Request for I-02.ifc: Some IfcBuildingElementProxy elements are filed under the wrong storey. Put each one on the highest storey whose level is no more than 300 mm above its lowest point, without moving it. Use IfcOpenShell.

First a look at what the model holds.

```python
import ifcopenshell
import ifcopenshell.util.element
import ifcopenshell.util.placement

model = ifcopenshell.open("I-02.ifc")
print(model.schema)
for storey in model.by_type("IfcBuildingStorey"):
    level = ifcopenshell.util.placement.get_storey_elevation(storey)
    count = sum(e.is_a("IfcBuildingElementProxy") for e in ifcopenshell.util.element.get_contained(storey))
    print(storey.id(), storey.Name, round(level, 3), count, sep=" | ")
```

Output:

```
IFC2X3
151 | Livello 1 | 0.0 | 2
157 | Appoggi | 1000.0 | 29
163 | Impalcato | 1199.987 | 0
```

```python
import ifcopenshell
import ifcopenshell.api.spatial
import ifcopenshell.geom
import ifcopenshell.util.element
import ifcopenshell.util.placement
import ifcopenshell.util.shape
import ifcopenshell.util.unit

model = ifcopenshell.open("I-02.ifc")
unit_scale = ifcopenshell.util.unit.calculate_unit_scale(model)
settings = ifcopenshell.geom.settings()

levels = sorted(
    ((ifcopenshell.util.placement.get_storey_elevation(s) * unit_scale, s) for s in model.by_type("IfcBuildingStorey")),
    key=lambda pair: pair[0],
)

for e in model.by_type("IfcBuildingElementProxy"):
    current = e.ContainedInStructure[0].RelatingStructure if e.ContainedInStructure else None
    if current is None or not current.is_a("IfcBuildingStorey"):
        continue
    shape = ifcopenshell.geom.create_shape(settings, e)
    bottom = ifcopenshell.util.shape.get_shape_bottom_elevation(shape, shape.geometry)
    below = [s for level, s in levels if level <= bottom + 0.3]
    storey = below[-1] if below else levels[0][1]
    if storey != current:
        # assign_container keeps the world position.
        ifcopenshell.api.spatial.assign_container(model, products=[e], relating_structure=storey)
        print(e.id(), current.Name, "->", storey.Name)

model.write("I-02_edited.ifc")
```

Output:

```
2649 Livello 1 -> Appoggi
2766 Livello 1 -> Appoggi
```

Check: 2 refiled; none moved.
